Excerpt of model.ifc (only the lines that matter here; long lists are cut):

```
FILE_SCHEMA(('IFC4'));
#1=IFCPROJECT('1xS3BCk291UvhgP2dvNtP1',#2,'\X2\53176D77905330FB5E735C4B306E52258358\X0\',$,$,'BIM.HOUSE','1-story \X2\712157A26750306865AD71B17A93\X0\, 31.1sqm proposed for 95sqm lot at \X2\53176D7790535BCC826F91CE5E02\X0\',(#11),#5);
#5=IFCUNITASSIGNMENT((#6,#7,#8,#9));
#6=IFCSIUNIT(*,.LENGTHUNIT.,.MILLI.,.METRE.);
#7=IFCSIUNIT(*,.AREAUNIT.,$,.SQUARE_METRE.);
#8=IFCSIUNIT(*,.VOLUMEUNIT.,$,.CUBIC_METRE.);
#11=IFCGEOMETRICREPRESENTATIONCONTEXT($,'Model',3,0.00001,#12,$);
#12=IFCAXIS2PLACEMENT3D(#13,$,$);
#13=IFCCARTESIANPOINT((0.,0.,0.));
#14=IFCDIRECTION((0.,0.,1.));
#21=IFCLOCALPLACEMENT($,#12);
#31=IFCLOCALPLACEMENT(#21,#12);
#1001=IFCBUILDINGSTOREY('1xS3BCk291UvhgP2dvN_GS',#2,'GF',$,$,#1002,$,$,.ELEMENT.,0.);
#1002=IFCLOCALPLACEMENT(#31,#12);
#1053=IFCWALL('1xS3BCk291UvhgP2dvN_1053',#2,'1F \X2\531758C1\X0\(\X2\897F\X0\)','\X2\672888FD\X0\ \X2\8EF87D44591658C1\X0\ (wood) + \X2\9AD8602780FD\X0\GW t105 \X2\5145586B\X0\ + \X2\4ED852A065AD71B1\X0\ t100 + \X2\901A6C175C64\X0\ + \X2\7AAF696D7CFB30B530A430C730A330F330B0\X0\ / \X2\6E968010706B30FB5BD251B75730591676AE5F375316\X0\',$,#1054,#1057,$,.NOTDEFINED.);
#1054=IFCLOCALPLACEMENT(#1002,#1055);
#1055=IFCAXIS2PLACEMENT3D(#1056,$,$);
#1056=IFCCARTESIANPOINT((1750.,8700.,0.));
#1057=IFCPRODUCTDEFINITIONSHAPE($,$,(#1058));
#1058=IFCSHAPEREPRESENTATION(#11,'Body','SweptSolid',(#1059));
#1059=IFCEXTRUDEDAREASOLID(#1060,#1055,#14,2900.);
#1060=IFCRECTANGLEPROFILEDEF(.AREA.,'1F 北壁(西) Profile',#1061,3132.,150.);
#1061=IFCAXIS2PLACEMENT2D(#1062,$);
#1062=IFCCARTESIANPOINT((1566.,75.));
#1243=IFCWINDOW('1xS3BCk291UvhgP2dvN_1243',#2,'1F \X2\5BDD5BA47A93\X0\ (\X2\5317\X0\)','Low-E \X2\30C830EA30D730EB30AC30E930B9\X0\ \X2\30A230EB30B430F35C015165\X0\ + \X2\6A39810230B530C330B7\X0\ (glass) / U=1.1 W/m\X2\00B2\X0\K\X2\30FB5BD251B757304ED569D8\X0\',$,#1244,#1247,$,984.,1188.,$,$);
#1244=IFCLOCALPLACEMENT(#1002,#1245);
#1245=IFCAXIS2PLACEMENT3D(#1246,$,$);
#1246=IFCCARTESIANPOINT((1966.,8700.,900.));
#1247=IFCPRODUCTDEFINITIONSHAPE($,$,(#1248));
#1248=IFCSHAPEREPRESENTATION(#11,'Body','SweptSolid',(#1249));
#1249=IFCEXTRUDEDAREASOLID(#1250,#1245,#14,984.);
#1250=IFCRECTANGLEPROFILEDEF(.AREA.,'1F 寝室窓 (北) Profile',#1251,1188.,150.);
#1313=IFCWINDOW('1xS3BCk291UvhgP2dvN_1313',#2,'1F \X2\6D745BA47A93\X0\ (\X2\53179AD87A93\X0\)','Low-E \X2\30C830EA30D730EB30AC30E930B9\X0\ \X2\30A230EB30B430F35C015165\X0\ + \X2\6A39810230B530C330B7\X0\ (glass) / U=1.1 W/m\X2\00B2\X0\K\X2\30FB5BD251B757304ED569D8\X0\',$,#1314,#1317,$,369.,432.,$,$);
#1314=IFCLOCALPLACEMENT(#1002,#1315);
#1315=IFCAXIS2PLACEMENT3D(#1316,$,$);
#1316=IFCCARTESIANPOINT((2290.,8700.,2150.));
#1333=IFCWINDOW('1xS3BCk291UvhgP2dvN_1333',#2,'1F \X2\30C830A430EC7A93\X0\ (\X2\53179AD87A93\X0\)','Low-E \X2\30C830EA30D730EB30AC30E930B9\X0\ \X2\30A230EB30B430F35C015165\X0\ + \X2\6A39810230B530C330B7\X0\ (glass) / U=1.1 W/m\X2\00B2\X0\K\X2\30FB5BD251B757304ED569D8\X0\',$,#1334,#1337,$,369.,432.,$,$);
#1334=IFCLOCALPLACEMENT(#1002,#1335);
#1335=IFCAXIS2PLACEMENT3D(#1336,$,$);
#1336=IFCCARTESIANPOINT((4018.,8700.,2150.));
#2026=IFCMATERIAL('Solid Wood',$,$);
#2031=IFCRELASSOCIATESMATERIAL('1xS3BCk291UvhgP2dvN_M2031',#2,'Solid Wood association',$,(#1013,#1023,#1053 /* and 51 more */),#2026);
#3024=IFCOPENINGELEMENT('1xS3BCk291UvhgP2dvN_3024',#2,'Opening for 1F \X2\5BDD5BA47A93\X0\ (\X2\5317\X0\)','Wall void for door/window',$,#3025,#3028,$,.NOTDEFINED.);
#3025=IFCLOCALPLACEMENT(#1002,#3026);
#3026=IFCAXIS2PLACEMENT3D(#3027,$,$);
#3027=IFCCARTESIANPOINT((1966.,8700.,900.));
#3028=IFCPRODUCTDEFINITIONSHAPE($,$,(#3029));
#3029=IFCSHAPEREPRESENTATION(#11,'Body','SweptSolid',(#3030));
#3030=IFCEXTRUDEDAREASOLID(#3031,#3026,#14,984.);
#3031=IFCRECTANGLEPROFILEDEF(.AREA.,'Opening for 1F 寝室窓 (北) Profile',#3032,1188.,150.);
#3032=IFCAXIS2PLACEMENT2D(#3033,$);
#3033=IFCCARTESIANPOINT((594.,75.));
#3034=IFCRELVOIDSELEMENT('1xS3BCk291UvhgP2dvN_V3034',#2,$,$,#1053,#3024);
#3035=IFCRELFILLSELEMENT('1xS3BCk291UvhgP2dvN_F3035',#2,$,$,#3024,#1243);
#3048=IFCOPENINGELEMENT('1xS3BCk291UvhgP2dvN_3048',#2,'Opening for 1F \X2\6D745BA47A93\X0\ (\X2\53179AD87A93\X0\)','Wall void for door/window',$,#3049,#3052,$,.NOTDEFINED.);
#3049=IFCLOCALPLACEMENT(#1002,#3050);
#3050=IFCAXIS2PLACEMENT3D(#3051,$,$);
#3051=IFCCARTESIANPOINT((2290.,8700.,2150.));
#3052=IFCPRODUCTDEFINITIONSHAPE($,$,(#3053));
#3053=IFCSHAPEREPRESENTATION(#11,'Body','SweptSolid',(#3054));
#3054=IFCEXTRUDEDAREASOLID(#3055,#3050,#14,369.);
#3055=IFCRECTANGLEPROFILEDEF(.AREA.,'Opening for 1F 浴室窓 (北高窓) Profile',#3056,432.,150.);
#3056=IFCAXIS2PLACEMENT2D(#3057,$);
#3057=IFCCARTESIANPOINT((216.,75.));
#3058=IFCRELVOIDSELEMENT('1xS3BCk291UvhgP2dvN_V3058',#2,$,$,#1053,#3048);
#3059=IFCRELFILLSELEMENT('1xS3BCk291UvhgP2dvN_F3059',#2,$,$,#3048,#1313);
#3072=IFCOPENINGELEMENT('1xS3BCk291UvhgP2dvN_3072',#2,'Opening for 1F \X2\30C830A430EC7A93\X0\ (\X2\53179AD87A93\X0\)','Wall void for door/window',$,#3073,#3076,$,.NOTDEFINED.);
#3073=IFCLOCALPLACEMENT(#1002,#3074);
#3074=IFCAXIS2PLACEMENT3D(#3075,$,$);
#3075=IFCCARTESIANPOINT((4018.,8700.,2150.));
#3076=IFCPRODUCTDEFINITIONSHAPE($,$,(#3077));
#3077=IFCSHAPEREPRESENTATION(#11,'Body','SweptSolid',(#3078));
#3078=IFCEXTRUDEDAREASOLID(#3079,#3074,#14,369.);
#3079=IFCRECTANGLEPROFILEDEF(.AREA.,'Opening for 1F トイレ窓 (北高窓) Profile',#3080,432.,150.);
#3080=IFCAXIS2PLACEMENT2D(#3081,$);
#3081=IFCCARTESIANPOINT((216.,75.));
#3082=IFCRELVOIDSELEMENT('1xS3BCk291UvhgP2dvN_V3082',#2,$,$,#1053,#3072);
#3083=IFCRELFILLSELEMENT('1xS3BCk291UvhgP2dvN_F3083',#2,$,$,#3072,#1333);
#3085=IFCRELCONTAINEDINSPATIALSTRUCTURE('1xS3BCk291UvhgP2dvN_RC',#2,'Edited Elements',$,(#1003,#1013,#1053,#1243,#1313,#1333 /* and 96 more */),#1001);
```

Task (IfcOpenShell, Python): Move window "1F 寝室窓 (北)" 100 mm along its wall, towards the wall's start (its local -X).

```python
import ifcopenshell
import ifcopenshell.api.geometry
import ifcopenshell.util.placement

model = ifcopenshell.open("model.ifc")

window = model.by_guid("1xS3BCk291UvhgP2dvN_1243")
opening = window.FillsVoids[0].RelatingOpeningElement
wall = opening.VoidsElements[0].RelatingBuildingElement

wall_matrix = ifcopenshell.util.placement.get_local_placement(wall.ObjectPlacement)
shift = wall_matrix[:3, 0] * -100.0
before = ifcopenshell.util.placement.get_local_placement(window.ObjectPlacement)[:3, 3].copy()

# The window is not placed relative to its opening, so move both.
for product in (opening, window):
    matrix = ifcopenshell.util.placement.get_local_placement(product.ObjectPlacement)
    matrix[:3, 3] += shift
    ifcopenshell.api.geometry.edit_object_placement(model, product=product, matrix=matrix, is_si=False)

after = ifcopenshell.util.placement.get_local_placement(window.ObjectPlacement)[:3, 3]
print("window moved by", (after - before).round(3) + 0.0)

model.write("model_edited.ifc")
```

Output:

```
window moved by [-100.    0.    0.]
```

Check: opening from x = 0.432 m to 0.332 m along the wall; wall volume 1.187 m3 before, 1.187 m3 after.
